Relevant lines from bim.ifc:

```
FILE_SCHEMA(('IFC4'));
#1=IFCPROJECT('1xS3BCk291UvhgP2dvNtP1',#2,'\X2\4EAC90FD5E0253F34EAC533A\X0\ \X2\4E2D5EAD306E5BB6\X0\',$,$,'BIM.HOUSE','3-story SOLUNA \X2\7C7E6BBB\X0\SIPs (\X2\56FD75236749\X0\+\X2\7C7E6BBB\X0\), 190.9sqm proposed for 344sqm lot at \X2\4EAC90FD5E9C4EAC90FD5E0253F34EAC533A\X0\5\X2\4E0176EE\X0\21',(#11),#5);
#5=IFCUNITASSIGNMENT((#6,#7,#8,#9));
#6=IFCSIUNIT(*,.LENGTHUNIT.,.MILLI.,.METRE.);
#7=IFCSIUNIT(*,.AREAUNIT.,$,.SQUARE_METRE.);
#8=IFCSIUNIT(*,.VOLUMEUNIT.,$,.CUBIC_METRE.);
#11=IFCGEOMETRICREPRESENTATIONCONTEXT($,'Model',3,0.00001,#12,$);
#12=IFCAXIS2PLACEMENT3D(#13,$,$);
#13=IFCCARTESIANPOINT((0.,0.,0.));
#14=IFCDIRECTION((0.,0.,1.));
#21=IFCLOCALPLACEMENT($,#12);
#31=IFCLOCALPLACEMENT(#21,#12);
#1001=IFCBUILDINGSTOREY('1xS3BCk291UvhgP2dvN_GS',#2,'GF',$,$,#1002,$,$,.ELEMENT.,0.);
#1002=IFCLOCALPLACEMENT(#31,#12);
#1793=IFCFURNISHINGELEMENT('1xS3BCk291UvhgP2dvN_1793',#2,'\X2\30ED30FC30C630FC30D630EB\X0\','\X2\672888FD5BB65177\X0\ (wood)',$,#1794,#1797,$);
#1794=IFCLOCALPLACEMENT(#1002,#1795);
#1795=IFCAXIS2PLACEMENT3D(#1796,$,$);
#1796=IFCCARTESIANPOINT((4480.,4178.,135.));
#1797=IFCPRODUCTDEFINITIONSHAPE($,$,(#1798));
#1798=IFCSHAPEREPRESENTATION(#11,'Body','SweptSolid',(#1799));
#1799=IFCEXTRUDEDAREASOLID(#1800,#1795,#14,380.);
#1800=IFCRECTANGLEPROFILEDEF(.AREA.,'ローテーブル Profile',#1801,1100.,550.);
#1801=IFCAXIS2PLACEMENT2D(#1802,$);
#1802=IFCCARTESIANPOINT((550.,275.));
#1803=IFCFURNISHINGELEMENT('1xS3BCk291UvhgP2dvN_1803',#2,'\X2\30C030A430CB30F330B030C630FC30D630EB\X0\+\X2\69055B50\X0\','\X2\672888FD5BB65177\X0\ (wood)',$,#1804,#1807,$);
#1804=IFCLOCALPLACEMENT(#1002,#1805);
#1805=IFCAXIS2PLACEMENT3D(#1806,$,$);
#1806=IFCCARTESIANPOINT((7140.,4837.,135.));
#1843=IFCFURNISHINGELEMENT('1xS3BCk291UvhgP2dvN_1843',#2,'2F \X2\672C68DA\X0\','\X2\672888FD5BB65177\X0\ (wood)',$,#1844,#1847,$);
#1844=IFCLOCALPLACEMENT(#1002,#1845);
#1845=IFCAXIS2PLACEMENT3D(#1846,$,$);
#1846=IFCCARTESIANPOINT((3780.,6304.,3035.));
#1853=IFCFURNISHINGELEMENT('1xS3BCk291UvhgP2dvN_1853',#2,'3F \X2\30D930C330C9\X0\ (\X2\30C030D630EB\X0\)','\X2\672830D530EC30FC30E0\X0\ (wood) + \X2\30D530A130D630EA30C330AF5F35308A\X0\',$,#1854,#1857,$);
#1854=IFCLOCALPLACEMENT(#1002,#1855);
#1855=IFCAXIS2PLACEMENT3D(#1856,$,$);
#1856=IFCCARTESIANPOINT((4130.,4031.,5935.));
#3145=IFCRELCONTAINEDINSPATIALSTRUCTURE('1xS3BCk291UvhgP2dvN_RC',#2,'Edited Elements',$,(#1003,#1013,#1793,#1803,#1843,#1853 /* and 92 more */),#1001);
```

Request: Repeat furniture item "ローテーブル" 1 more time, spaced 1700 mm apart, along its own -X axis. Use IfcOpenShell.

```python
import ifcopenshell
import ifcopenshell.api.geometry
import ifcopenshell.api.root
import ifcopenshell.util.element
import ifcopenshell.util.placement

model = ifcopenshell.open("bim.ifc")


def reuse_history(source, copy):
    """copy_class also copies each property set's owner history, people and application; keep the originals."""
    for rel in copy.IsDefinedBy:
        if rel.is_a("IfcRelDefinesByProperties") and (history := rel.RelatingPropertyDefinition.OwnerHistory):
            rel.RelatingPropertyDefinition.OwnerHistory = source.OwnerHistory
            ifcopenshell.util.element.remove_deep2(model, history)


source = model.by_guid("1xS3BCk291UvhgP2dvN_1793")
base = ifcopenshell.util.placement.get_local_placement(source.ObjectPlacement)
step = -base[:3, 0] * 1700.0

for i in range(1, 2):
    copy = ifcopenshell.api.root.copy_class(model, product=source)
    copy.Representation = ifcopenshell.util.element.copy_deep(
        model, source.Representation, exclude=["IfcGeometricRepresentationContext", "IfcRepresentationMap"]
    )
    reuse_history(source, copy)
    matrix = base.copy()
    matrix[:3, 3] += i * step
    print("added at", matrix[:3, 3].round(3) + 0.0)
    ifcopenshell.api.geometry.edit_object_placement(model, product=copy, matrix=matrix, is_si=False)

model.write("bim-out.ifc")
```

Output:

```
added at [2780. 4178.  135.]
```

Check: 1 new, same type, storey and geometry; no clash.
